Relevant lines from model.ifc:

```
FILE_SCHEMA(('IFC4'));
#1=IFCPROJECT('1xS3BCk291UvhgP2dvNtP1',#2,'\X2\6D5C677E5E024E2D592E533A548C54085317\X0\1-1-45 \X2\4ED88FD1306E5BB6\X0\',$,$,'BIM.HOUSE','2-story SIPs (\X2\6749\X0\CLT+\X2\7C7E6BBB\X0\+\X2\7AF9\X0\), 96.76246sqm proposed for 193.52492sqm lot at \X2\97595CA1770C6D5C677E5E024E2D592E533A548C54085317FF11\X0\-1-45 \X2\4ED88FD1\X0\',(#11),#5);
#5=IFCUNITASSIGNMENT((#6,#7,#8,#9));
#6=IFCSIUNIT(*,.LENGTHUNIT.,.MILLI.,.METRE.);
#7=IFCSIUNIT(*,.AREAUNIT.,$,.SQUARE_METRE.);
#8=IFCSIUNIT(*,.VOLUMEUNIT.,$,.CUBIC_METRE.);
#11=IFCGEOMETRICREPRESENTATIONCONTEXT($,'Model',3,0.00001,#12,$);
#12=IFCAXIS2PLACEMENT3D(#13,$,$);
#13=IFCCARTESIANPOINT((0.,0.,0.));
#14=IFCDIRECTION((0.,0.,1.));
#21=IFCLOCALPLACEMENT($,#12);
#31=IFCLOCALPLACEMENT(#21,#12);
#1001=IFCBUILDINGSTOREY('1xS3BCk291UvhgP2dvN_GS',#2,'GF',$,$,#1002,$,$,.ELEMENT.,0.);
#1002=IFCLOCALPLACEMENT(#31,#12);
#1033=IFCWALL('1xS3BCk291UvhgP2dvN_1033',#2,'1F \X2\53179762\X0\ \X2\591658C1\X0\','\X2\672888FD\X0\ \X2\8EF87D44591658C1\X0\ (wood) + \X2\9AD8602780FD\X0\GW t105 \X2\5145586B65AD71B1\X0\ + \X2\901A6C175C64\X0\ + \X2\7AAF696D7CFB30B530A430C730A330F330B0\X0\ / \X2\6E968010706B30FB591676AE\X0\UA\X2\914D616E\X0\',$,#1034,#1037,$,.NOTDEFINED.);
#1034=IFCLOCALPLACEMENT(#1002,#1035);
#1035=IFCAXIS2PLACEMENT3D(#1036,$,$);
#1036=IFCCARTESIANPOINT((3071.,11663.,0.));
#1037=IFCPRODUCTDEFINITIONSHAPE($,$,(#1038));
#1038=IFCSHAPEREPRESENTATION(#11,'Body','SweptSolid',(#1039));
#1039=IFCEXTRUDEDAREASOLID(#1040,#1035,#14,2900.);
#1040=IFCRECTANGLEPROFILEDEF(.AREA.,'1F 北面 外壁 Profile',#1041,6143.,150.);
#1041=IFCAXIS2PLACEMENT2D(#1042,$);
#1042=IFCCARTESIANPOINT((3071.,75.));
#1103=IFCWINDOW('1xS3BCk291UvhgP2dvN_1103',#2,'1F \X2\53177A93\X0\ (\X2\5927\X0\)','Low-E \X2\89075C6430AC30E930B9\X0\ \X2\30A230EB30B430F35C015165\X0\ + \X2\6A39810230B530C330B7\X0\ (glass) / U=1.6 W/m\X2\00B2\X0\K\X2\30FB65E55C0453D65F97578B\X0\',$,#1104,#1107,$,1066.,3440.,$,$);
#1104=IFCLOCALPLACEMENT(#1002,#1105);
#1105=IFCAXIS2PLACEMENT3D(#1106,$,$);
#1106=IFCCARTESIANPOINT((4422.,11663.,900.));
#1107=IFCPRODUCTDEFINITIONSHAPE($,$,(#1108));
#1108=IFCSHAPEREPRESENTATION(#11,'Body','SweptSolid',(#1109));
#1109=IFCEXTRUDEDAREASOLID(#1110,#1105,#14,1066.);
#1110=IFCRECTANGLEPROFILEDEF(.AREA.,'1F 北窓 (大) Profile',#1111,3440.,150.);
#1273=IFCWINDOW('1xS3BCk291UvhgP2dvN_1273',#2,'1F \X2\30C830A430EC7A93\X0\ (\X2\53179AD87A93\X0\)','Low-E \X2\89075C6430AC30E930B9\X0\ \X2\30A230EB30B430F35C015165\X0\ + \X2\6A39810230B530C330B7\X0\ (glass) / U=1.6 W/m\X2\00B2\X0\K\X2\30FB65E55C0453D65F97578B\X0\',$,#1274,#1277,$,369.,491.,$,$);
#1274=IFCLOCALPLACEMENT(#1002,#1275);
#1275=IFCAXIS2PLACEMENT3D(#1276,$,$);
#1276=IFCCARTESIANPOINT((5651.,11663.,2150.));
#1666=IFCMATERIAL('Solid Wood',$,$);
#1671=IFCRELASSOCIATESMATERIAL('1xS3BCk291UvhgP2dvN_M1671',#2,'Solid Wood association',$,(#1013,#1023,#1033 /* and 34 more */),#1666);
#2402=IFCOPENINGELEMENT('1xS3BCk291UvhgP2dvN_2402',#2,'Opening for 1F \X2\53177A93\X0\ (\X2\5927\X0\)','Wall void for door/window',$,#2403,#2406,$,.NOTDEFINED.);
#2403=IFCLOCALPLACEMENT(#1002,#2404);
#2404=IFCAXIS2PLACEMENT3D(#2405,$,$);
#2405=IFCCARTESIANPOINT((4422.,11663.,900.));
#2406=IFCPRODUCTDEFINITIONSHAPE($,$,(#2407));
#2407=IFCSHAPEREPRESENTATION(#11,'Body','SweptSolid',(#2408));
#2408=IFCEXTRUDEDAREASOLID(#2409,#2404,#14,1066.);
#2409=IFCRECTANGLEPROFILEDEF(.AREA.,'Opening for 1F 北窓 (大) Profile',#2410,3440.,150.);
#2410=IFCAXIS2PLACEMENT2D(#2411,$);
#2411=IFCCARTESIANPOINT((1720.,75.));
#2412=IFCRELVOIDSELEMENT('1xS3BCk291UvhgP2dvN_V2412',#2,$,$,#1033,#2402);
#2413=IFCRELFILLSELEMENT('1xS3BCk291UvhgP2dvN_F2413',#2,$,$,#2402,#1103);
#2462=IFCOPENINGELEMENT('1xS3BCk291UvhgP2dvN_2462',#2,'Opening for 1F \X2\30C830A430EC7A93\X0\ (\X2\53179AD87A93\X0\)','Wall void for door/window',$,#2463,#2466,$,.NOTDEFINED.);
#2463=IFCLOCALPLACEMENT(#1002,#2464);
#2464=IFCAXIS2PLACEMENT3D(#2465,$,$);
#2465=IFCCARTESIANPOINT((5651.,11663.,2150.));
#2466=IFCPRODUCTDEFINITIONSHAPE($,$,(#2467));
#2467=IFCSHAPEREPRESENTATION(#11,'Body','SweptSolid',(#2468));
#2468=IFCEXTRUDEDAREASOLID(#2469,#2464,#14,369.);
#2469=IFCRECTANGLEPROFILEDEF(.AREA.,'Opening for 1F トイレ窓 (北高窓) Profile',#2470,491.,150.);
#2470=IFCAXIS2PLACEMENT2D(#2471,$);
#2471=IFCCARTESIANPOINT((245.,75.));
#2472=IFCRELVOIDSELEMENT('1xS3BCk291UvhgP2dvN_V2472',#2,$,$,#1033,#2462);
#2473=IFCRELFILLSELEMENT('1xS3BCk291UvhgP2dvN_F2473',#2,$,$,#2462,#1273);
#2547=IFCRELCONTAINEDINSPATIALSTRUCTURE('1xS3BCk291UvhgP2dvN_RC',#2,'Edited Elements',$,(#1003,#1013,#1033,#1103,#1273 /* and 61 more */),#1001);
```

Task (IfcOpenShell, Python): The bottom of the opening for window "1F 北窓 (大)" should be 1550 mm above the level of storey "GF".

```python
import numpy as np
import ifcopenshell
import ifcopenshell.api.geometry
import ifcopenshell.geom
import ifcopenshell.util.element
import ifcopenshell.util.placement
import ifcopenshell.util.shape
import ifcopenshell.util.unit

model = ifcopenshell.open("model.ifc")
unit_scale = ifcopenshell.util.unit.calculate_unit_scale(model)

window = model.by_guid("1xS3BCk291UvhgP2dvN_1103")
opening = window.FillsVoids[0].RelatingOpeningElement
storey = ifcopenshell.util.element.get_container(window, ifc_class="IfcBuildingStorey")
level = ifcopenshell.util.placement.get_local_placement(storey.ObjectPlacement)[2, 3]

# The opening's origin need not be at the sill, so measure its lowest point.
shape = ifcopenshell.geom.create_shape(ifcopenshell.geom.settings(), opening)
bottom = ifcopenshell.util.shape.get_shape_bottom_elevation(shape, shape.geometry) / unit_scale
dz = level + 1.55 / unit_scale - bottom

shift = np.array([0.0, 0.0, dz])
# The window is not placed relative to its opening, so move both.
for product in (opening, window):
    matrix = ifcopenshell.util.placement.get_local_placement(product.ObjectPlacement)
    matrix[:3, 3] += shift
    ifcopenshell.api.geometry.edit_object_placement(model, product=product, matrix=matrix, is_si=False)

print(f"moved by {dz * unit_scale:+.3f} m")

model.write("model_updated.ifc")
```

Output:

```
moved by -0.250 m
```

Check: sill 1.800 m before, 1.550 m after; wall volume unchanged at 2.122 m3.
